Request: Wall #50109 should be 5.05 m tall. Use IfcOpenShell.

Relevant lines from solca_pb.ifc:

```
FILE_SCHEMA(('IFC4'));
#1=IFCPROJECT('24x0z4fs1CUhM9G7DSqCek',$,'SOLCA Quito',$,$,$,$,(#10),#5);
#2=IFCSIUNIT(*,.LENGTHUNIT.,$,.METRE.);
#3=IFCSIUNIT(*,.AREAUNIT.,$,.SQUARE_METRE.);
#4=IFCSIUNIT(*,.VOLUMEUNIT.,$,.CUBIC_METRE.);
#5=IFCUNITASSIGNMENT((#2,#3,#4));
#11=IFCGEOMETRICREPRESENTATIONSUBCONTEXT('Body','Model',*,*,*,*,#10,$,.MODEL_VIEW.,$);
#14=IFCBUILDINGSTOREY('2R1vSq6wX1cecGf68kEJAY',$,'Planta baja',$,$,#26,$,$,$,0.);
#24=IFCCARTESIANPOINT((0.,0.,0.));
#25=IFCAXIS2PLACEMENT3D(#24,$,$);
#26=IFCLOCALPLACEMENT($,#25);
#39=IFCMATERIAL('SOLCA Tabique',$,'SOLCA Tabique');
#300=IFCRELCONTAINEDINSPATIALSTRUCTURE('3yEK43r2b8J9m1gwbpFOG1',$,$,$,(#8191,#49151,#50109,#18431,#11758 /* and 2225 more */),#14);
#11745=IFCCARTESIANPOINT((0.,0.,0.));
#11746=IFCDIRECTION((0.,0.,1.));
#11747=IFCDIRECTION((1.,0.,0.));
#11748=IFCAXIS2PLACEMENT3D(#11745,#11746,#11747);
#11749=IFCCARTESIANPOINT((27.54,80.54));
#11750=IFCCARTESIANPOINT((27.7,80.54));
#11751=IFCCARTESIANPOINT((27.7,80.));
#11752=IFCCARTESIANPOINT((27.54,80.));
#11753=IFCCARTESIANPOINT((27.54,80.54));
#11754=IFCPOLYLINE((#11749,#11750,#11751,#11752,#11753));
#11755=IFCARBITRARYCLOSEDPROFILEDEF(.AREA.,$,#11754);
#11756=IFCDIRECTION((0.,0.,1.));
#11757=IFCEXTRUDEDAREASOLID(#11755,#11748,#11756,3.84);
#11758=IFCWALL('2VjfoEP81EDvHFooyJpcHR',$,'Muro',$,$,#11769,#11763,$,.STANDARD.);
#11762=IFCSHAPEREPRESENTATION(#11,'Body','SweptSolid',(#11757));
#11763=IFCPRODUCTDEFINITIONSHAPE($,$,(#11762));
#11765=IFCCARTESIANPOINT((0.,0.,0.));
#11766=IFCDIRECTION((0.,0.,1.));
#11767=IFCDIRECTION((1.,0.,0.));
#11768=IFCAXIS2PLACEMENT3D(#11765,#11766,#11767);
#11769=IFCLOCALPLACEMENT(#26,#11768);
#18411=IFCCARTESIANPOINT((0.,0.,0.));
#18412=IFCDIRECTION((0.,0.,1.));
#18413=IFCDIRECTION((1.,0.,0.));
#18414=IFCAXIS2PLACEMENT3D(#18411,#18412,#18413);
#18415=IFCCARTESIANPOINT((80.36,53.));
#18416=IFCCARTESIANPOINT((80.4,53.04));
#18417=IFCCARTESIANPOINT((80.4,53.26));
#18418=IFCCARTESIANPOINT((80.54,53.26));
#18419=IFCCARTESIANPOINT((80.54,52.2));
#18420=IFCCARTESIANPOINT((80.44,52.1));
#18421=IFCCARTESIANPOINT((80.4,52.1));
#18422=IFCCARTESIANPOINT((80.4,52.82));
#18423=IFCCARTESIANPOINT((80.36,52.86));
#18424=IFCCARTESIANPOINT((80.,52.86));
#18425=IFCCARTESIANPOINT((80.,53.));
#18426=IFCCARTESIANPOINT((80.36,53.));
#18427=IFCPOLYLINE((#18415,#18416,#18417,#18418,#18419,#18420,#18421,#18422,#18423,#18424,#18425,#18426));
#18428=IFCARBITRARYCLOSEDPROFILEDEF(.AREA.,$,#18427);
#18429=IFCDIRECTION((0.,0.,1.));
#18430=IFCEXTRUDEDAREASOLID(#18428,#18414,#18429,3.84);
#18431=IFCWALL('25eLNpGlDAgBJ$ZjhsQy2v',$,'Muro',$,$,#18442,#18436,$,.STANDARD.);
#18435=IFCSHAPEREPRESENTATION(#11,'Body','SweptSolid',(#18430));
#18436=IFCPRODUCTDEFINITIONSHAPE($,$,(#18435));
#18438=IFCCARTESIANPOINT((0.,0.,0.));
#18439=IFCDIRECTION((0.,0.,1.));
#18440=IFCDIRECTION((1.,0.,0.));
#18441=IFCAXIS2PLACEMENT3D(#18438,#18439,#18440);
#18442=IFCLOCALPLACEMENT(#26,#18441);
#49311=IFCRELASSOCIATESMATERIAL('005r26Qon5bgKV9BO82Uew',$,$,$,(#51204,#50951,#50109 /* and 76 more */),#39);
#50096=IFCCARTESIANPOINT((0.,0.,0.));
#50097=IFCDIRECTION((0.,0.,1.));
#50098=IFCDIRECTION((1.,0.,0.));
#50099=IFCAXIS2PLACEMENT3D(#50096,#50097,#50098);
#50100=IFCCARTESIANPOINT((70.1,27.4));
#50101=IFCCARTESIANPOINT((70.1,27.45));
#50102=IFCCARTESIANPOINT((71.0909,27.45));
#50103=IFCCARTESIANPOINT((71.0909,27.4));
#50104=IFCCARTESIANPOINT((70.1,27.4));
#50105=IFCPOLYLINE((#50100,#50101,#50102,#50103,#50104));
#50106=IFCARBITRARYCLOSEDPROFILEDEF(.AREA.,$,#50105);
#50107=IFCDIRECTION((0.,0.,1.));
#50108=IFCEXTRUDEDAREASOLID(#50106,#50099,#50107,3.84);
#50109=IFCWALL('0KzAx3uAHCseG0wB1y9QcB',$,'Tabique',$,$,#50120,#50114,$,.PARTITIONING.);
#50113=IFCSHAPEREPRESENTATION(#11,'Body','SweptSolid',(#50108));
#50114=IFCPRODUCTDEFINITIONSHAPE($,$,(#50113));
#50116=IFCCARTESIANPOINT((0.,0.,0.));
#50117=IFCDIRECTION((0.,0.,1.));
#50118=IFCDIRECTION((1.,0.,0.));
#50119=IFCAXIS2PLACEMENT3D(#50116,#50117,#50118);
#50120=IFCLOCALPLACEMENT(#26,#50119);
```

```python
import ifcopenshell
import ifcopenshell.geom
import ifcopenshell.util.representation
import ifcopenshell.util.shape
import ifcopenshell.util.unit

model = ifcopenshell.open("solca_pb.ifc")
unit_scale = ifcopenshell.util.unit.calculate_unit_scale(model)
settings = ifcopenshell.geom.settings()


def volume(element):
    """Net volume in cubic metres, openings subtracted."""
    shape = ifcopenshell.geom.create_shape(settings, element)
    return ifcopenshell.util.shape.get_volume(shape.geometry)


wall = model.by_guid("0KzAx3uAHCseG0wB1y9QcB")
before = volume(wall)

body = ifcopenshell.util.representation.get_representation(wall, "Model", "Body")
solid = body.Items[0]
old_height = solid.Depth
solid.Depth = 5.05 / unit_scale
after = volume(wall)

print(f"height {old_height:g} -> {solid.Depth:g}, volume {before:.3f} -> {after:.3f} m3")

model.write("solca_pb-out.ifc")
```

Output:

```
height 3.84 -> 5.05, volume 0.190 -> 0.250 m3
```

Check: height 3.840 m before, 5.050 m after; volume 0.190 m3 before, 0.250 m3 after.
